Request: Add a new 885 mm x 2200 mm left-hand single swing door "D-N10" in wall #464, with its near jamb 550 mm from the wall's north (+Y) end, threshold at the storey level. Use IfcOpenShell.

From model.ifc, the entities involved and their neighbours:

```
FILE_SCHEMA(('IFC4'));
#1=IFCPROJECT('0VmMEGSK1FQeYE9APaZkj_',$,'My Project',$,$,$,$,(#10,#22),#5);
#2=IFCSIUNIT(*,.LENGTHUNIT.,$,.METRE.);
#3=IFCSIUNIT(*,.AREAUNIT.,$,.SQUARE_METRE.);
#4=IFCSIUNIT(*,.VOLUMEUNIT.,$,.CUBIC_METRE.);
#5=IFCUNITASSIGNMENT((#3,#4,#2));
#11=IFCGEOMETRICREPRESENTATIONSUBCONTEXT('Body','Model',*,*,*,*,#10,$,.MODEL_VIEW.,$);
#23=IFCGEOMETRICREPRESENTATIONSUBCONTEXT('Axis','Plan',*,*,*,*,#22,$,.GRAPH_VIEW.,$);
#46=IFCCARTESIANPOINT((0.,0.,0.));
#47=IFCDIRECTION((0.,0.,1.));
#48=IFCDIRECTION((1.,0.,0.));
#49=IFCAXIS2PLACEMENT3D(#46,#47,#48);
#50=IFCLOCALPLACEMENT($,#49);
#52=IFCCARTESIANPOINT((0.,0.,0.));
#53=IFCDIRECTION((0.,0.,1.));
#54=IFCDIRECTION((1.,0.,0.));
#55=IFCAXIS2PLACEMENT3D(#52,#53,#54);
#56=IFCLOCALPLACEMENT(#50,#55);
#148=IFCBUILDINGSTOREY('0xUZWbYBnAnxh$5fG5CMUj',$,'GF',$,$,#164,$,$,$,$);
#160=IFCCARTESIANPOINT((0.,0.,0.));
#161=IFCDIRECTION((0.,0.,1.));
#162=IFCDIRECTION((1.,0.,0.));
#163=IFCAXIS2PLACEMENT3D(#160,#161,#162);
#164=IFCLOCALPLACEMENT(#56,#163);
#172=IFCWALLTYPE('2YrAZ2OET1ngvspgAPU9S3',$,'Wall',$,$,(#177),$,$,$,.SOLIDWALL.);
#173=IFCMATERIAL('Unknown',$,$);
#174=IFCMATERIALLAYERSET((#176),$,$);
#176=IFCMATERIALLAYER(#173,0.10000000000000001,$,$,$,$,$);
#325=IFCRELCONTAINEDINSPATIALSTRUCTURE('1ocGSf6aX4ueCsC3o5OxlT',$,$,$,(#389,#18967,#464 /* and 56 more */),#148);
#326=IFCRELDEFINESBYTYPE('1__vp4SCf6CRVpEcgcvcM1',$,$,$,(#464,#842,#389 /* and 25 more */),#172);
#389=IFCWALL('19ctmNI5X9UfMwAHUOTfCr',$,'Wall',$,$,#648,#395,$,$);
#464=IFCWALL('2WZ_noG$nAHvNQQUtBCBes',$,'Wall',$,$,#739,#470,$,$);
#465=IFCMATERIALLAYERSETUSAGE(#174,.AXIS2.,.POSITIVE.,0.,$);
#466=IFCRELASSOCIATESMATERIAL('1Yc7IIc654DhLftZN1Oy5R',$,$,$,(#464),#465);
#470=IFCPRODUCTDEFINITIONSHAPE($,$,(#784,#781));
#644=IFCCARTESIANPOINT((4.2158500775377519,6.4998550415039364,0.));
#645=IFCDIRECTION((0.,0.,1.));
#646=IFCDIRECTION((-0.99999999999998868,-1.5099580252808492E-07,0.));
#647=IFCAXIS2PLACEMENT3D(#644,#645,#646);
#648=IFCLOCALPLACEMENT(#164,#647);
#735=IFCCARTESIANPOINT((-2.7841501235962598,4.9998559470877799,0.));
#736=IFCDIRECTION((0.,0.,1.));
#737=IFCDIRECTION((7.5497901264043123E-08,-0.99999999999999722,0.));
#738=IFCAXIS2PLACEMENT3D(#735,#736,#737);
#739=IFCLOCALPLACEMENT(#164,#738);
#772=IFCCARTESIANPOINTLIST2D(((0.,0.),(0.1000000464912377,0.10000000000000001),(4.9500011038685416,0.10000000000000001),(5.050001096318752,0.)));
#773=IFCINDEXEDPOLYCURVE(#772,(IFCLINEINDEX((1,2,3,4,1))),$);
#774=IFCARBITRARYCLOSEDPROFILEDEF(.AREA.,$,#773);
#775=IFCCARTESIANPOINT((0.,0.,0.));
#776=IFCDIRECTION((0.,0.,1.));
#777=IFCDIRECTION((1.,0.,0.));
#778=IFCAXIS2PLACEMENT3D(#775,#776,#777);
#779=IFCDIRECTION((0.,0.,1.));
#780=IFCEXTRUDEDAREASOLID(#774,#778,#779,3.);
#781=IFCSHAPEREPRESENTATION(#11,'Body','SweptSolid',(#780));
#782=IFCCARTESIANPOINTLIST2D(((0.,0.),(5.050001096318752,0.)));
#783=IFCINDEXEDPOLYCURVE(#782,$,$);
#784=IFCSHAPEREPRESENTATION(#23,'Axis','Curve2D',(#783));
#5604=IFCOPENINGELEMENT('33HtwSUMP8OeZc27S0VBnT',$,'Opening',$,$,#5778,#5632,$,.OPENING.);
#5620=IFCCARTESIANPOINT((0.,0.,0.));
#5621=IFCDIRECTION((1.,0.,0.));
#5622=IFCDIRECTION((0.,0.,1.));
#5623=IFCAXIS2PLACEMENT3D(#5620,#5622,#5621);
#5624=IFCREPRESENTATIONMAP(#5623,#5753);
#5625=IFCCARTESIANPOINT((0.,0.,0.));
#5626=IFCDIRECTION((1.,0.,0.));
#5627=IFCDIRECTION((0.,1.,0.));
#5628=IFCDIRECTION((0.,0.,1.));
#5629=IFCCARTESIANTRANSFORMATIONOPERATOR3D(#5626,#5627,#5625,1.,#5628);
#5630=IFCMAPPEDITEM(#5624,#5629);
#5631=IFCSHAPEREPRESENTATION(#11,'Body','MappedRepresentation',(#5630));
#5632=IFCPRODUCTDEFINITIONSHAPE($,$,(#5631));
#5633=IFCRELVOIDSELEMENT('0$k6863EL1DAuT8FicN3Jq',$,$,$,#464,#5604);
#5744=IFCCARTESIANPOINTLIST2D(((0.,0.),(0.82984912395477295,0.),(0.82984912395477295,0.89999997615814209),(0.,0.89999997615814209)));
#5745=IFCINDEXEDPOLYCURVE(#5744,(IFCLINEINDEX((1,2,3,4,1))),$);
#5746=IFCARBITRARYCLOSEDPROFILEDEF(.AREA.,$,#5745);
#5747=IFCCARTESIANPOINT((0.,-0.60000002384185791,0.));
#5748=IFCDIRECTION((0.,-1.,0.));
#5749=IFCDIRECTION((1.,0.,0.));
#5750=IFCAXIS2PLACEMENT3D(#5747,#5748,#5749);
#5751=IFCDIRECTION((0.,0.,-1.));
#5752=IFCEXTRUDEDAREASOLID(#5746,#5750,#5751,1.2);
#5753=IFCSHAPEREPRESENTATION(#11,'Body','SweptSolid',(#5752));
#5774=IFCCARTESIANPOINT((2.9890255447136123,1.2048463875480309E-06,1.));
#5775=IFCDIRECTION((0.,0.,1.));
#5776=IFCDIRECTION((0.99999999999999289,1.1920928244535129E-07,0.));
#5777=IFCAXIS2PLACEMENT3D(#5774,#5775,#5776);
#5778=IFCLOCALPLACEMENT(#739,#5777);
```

```python
import numpy as np
import ifcopenshell
import ifcopenshell.api.feature
import ifcopenshell.api.geometry
import ifcopenshell.api.root
import ifcopenshell.api.spatial
import ifcopenshell.geom
import ifcopenshell.util.element
import ifcopenshell.util.placement
import ifcopenshell.util.representation
import ifcopenshell.util.shape
import ifcopenshell.util.unit

model = ifcopenshell.open("model.ifc")
unit_scale = ifcopenshell.util.unit.calculate_unit_scale(model)
settings = ifcopenshell.geom.settings()


def volume(element):
    """Net volume in cubic metres, openings subtracted."""
    shape = ifcopenshell.geom.create_shape(settings, element)
    return ifcopenshell.util.shape.get_volume(shape.geometry)


wall = model.by_guid("2WZ_noG$nAHvNQQUtBCBes")
storey = ifcopenshell.util.element.get_container(wall, ifc_class="IfcBuildingStorey")
context = ifcopenshell.util.representation.get_context(model, "Model", "Body", "MODEL_VIEW")
before = volume(wall)

width, height, from_end, sill = 0.885, 2.2, 0.55, 0.0  # metres

# The wall runs along its own X axis, and the end named is its -X end.
wall_shape = ifcopenshell.geom.create_shape(settings, wall)
x, y, z = ifcopenshell.util.shape.get_vertices(wall_shape.geometry).T
start = x.min() + from_end
face, thickness = float(y.min()), float(y.max() - y.min())
wall_matrix = ifcopenshell.util.placement.get_local_placement(wall.ObjectPlacement)
level = ifcopenshell.util.placement.get_local_placement(storey.ObjectPlacement)[2, 3]


def in_wall(x, y):
    """Placement at x, y metres in the wall's axes, at sill height."""
    matrix = wall_matrix.copy()
    matrix[:, 3] = wall_matrix @ np.array([x / unit_scale, y / unit_scale, 0.0, 1.0])
    matrix[2, 3] = level + sill / unit_scale
    return matrix


# Opening: a box that overshoots both wall faces by 50 mm.
opening = ifcopenshell.api.root.create_entity(model, ifc_class="IfcOpeningElement", predefined_type="OPENING")
box = ifcopenshell.api.geometry.add_wall_representation(
    model, context=context, length=width, height=height, thickness=thickness + 0.1
)
ifcopenshell.api.geometry.assign_representation(model, product=opening, representation=box)
ifcopenshell.api.geometry.edit_object_placement(model, product=opening, matrix=in_wall(start, face - 0.05), is_si=False)
ifcopenshell.api.feature.add_feature(model, feature=opening, element=wall)

door = ifcopenshell.api.root.create_entity(model, ifc_class="IfcDoor", name="D-N10", predefined_type="DOOR")
door.OverallWidth, door.OverallHeight = width / unit_scale, height / unit_scale
door.OperationType = "SINGLE_SWING_LEFT"
body = ifcopenshell.api.geometry.add_door_representation(
    model,
    context=context,
    overall_width=door.OverallWidth,
    overall_height=door.OverallHeight,
    operation_type="SINGLE_SWING_LEFT",
    lining_properties={"LiningDepth": thickness / unit_scale, "ThresholdDepth": thickness / unit_scale},
)
ifcopenshell.api.geometry.assign_representation(model, product=door, representation=body)
ifcopenshell.api.spatial.assign_container(model, products=[door], relating_structure=storey)
ifcopenshell.api.feature.add_filling(model, opening=opening, element=door)

# The lining spans the wall, so the door starts at the wall face.
ifcopenshell.api.geometry.edit_object_placement(model, product=door, matrix=in_wall(start, face), is_si=False)

after = volume(wall)

print(f"wall volume {before:.3f} -> {after:.3f} m3")

model.write("model_edited.ifc")
```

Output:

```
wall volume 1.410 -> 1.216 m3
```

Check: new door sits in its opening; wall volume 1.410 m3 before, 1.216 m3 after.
